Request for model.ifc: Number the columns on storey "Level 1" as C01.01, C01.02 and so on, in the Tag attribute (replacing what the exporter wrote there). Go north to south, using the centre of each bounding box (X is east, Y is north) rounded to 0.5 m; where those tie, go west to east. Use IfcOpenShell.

First a look at what the model holds.

```python
import ifcopenshell
import ifcopenshell.util.element
import ifcopenshell.util.placement

model = ifcopenshell.open("model.ifc")
print(model.schema)
storey = next(s for s in model.by_type("IfcBuildingStorey") if s.Name == "Level 1")
columns = [e for e in ifcopenshell.util.element.get_decomposition(storey) if e.is_a("IfcColumn")]
for e in sorted(columns, key=lambda e: e.id()):
    origin = ifcopenshell.util.placement.get_local_placement(e.ObjectPlacement)[:3, 3]
    print(e.id(), e.Tag, e.Name, origin.round(2) + 0.0, sep=" | ")
```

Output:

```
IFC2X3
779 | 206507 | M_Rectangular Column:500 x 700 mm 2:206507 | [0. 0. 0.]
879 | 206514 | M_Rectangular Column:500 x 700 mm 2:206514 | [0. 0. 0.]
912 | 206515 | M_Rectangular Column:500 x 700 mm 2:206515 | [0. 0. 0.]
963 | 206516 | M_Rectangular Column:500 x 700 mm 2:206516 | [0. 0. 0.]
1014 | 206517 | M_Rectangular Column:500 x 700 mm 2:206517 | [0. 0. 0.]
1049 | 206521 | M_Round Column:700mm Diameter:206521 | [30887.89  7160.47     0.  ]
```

```python
import ifcopenshell
import ifcopenshell.geom
import ifcopenshell.util.element
import ifcopenshell.util.shape

model = ifcopenshell.open("model.ifc")
settings = ifcopenshell.geom.settings()
settings.set("use-world-coords", True)


def centre(element):
    shape = ifcopenshell.geom.create_shape(settings, element)
    return ifcopenshell.util.shape.get_bbox_centroid(shape.geometry)


storey = next(s for s in model.by_type("IfcBuildingStorey") if s.Name == "Level 1")
columns = [e for e in ifcopenshell.util.element.get_decomposition(storey) if e.is_a("IfcColumn")]

# Insertion points can sit at a corner or the storey origin, so sort by the geometry (in metres).
centres = {e: centre(e) for e in columns}
columns.sort(key=lambda e: (-round(centres[e][1] / 0.5), centres[e][0]))

for i, e in enumerate(columns, start=1):
    number = f"C01.{i:02d}"
    e.Tag = number
    print(e.id(), number)

model.write("model-out.ifc")
```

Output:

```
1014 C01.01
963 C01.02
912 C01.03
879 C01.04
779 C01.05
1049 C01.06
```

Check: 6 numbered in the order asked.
